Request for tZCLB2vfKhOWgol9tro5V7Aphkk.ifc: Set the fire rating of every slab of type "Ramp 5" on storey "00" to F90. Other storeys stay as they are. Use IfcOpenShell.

First a look at what the model holds.

```python
import ifcopenshell
import ifcopenshell.util.element

model = ifcopenshell.open("tZCLB2vfKhOWgol9tro5V7Aphkk.ifc")
print(model.schema)
storey = next(s for s in model.by_type("IfcBuildingStorey") if s.Name == "00")
slabs = [e for e in ifcopenshell.util.element.get_decomposition(storey) if e.is_a("IfcSlab")]
seen = {}
for e in slabs:
    element_type = ifcopenshell.util.element.get_type(e)
    key = (element_type.Name if element_type != e and element_type else None, ifcopenshell.util.element.get_pset(e, "Pset_SlabCommon", "FireRating"))
    seen[key] = seen.get(key, 0) + 1
for (name, value), count in sorted(seen.items(), key=str):
    print(count, "x", name, "|", value)
```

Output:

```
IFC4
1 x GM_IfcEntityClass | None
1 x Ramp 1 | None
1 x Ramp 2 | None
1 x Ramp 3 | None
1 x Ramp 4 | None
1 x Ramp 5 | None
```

```python
import ifcopenshell
import ifcopenshell.api.pset
import ifcopenshell.util.element

model = ifcopenshell.open("tZCLB2vfKhOWgol9tro5V7Aphkk.ifc")

storey = next(s for s in model.by_type("IfcBuildingStorey") if s.Name == "00")
slabs = [e for e in ifcopenshell.util.element.get_decomposition(storey) if e.is_a("IfcSlab")]

count = 0
for e in slabs:
    element_type = ifcopenshell.util.element.get_type(e)
    if element_type in (None, e) or element_type.Name != "Ramp 5":
        continue
    # add_pset returns the element's existing set when there is one.
    pset = ifcopenshell.api.pset.add_pset(model, product=e, name="Pset_SlabCommon")
    ifcopenshell.api.pset.edit_pset(model, pset=pset, properties={"FireRating": "F90"})
    count += 1

print(count, "slabs updated")

model.write("tZCLB2vfKhOWgol9tro5V7Aphkk_rev.ifc")
```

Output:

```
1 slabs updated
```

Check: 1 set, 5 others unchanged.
